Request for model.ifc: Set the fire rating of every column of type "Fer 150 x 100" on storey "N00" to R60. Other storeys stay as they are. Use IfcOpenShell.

First a look at what the model holds.

```python
import ifcopenshell
import ifcopenshell.util.element

model = ifcopenshell.open("model.ifc")
print(model.schema)
storey = next(s for s in model.by_type("IfcBuildingStorey") if s.Name == "N00")
columns = [e for e in ifcopenshell.util.element.get_decomposition(storey) if e.is_a("IfcColumn")]
seen = {}
for e in columns:
    element_type = ifcopenshell.util.element.get_type(e)
    key = (element_type.Name if element_type != e and element_type else None, ifcopenshell.util.element.get_pset(e, "Pset_ColumnCommon", "FireRating"))
    seen[key] = seen.get(key, 0) + 1
for (name, value), count in sorted(seen.items(), key=str):
    print(count, "x", name, "|", value)
```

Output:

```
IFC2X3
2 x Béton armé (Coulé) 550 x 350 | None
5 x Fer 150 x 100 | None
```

```python
import ifcopenshell
import ifcopenshell.api.pset
import ifcopenshell.util.element

model = ifcopenshell.open("model.ifc")

storey = next(s for s in model.by_type("IfcBuildingStorey") if s.Name == "N00")
columns = [e for e in ifcopenshell.util.element.get_decomposition(storey) if e.is_a("IfcColumn")]

count = 0
for e in columns:
    element_type = ifcopenshell.util.element.get_type(e)
    if element_type in (None, e) or element_type.Name != "Fer 150 x 100":
        continue
    # add_pset returns the element's existing set when there is one.
    pset = ifcopenshell.api.pset.add_pset(model, product=e, name="Pset_ColumnCommon")
    ifcopenshell.api.pset.edit_pset(model, pset=pset, properties={"FireRating": "R60"})
    count += 1

print(count, "columns updated")

model.write("model_edited.ifc")
```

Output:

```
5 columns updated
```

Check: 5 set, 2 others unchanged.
